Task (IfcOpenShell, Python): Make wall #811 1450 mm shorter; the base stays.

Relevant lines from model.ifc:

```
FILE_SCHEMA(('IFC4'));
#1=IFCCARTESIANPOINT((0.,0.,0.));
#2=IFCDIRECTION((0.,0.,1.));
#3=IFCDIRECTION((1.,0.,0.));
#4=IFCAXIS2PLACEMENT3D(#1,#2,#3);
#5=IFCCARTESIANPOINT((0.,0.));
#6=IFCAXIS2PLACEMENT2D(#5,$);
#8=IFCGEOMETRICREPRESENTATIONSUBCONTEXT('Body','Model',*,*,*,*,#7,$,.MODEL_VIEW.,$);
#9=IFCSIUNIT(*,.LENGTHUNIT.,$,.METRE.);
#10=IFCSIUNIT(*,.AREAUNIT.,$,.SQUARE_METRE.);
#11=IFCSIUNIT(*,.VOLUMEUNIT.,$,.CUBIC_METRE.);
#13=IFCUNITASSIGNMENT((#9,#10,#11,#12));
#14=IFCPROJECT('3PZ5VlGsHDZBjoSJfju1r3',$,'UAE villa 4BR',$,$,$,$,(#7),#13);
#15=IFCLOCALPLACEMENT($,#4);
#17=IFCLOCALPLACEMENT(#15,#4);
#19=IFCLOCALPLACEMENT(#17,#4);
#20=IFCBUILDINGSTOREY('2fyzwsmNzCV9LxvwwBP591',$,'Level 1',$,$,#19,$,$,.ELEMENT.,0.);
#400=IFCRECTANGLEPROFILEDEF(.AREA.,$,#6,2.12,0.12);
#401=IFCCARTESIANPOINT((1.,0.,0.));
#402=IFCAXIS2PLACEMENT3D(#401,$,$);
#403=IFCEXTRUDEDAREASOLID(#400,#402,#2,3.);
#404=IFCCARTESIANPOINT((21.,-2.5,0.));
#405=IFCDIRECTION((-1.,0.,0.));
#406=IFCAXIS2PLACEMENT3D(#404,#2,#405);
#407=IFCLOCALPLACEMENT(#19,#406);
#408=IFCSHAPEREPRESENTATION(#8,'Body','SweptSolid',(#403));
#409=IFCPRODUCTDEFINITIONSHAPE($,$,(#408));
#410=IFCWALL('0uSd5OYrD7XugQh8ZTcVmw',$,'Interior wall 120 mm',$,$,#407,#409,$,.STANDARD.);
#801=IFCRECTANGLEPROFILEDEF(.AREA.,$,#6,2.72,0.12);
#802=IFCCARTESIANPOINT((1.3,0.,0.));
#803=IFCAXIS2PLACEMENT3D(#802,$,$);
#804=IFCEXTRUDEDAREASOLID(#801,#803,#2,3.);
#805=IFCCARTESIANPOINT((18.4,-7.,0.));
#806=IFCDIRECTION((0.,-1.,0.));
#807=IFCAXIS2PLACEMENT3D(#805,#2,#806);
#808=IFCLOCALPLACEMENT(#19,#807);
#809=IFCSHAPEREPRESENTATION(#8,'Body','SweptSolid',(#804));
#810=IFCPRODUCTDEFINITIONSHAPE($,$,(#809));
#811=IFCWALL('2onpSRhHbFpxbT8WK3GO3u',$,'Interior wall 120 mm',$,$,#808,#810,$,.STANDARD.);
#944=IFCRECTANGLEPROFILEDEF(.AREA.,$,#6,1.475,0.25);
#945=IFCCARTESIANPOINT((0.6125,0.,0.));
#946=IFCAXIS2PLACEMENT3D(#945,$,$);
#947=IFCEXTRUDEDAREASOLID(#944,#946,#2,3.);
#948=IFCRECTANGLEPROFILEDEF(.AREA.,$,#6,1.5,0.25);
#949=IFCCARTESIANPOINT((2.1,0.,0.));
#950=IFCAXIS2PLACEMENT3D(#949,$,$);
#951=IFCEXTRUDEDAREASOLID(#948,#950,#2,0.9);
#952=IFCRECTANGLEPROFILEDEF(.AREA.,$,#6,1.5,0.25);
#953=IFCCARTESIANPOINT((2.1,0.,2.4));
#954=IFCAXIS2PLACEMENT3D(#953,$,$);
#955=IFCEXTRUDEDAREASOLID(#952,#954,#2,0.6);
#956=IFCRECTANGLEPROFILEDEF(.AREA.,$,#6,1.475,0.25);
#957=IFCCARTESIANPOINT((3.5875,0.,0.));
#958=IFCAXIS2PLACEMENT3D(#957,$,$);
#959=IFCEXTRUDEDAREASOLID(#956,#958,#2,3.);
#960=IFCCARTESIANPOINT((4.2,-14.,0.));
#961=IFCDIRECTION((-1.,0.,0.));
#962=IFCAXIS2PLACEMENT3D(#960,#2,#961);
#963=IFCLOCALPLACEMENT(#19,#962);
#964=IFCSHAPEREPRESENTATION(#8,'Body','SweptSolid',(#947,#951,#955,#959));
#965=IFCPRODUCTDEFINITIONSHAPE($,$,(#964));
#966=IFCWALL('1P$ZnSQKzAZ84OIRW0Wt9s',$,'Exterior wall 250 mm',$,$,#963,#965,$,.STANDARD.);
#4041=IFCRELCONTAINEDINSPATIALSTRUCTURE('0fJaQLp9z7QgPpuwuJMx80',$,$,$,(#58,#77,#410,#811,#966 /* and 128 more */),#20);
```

```python
import ifcopenshell
import ifcopenshell.geom
import ifcopenshell.util.representation
import ifcopenshell.util.shape
import ifcopenshell.util.unit

model = ifcopenshell.open("model.ifc")
unit_scale = ifcopenshell.util.unit.calculate_unit_scale(model)
settings = ifcopenshell.geom.settings()


def volume(element):
    """Net volume in cubic metres, openings subtracted."""
    shape = ifcopenshell.geom.create_shape(settings, element)
    return ifcopenshell.util.shape.get_volume(shape.geometry)


wall = model.by_guid("2onpSRhHbFpxbT8WK3GO3u")
before = volume(wall)

body = ifcopenshell.util.representation.get_representation(wall, "Model", "Body")
solid = body.Items[0]
old_height = solid.Depth
solid.Depth -= 1.45 / unit_scale
after = volume(wall)

print(f"height {old_height:g} -> {solid.Depth:g}, volume {before:.3f} -> {after:.3f} m3")

model.write("model_updated.ifc")
```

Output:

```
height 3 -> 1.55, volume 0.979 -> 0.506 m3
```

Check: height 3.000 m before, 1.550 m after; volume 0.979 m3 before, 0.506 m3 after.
